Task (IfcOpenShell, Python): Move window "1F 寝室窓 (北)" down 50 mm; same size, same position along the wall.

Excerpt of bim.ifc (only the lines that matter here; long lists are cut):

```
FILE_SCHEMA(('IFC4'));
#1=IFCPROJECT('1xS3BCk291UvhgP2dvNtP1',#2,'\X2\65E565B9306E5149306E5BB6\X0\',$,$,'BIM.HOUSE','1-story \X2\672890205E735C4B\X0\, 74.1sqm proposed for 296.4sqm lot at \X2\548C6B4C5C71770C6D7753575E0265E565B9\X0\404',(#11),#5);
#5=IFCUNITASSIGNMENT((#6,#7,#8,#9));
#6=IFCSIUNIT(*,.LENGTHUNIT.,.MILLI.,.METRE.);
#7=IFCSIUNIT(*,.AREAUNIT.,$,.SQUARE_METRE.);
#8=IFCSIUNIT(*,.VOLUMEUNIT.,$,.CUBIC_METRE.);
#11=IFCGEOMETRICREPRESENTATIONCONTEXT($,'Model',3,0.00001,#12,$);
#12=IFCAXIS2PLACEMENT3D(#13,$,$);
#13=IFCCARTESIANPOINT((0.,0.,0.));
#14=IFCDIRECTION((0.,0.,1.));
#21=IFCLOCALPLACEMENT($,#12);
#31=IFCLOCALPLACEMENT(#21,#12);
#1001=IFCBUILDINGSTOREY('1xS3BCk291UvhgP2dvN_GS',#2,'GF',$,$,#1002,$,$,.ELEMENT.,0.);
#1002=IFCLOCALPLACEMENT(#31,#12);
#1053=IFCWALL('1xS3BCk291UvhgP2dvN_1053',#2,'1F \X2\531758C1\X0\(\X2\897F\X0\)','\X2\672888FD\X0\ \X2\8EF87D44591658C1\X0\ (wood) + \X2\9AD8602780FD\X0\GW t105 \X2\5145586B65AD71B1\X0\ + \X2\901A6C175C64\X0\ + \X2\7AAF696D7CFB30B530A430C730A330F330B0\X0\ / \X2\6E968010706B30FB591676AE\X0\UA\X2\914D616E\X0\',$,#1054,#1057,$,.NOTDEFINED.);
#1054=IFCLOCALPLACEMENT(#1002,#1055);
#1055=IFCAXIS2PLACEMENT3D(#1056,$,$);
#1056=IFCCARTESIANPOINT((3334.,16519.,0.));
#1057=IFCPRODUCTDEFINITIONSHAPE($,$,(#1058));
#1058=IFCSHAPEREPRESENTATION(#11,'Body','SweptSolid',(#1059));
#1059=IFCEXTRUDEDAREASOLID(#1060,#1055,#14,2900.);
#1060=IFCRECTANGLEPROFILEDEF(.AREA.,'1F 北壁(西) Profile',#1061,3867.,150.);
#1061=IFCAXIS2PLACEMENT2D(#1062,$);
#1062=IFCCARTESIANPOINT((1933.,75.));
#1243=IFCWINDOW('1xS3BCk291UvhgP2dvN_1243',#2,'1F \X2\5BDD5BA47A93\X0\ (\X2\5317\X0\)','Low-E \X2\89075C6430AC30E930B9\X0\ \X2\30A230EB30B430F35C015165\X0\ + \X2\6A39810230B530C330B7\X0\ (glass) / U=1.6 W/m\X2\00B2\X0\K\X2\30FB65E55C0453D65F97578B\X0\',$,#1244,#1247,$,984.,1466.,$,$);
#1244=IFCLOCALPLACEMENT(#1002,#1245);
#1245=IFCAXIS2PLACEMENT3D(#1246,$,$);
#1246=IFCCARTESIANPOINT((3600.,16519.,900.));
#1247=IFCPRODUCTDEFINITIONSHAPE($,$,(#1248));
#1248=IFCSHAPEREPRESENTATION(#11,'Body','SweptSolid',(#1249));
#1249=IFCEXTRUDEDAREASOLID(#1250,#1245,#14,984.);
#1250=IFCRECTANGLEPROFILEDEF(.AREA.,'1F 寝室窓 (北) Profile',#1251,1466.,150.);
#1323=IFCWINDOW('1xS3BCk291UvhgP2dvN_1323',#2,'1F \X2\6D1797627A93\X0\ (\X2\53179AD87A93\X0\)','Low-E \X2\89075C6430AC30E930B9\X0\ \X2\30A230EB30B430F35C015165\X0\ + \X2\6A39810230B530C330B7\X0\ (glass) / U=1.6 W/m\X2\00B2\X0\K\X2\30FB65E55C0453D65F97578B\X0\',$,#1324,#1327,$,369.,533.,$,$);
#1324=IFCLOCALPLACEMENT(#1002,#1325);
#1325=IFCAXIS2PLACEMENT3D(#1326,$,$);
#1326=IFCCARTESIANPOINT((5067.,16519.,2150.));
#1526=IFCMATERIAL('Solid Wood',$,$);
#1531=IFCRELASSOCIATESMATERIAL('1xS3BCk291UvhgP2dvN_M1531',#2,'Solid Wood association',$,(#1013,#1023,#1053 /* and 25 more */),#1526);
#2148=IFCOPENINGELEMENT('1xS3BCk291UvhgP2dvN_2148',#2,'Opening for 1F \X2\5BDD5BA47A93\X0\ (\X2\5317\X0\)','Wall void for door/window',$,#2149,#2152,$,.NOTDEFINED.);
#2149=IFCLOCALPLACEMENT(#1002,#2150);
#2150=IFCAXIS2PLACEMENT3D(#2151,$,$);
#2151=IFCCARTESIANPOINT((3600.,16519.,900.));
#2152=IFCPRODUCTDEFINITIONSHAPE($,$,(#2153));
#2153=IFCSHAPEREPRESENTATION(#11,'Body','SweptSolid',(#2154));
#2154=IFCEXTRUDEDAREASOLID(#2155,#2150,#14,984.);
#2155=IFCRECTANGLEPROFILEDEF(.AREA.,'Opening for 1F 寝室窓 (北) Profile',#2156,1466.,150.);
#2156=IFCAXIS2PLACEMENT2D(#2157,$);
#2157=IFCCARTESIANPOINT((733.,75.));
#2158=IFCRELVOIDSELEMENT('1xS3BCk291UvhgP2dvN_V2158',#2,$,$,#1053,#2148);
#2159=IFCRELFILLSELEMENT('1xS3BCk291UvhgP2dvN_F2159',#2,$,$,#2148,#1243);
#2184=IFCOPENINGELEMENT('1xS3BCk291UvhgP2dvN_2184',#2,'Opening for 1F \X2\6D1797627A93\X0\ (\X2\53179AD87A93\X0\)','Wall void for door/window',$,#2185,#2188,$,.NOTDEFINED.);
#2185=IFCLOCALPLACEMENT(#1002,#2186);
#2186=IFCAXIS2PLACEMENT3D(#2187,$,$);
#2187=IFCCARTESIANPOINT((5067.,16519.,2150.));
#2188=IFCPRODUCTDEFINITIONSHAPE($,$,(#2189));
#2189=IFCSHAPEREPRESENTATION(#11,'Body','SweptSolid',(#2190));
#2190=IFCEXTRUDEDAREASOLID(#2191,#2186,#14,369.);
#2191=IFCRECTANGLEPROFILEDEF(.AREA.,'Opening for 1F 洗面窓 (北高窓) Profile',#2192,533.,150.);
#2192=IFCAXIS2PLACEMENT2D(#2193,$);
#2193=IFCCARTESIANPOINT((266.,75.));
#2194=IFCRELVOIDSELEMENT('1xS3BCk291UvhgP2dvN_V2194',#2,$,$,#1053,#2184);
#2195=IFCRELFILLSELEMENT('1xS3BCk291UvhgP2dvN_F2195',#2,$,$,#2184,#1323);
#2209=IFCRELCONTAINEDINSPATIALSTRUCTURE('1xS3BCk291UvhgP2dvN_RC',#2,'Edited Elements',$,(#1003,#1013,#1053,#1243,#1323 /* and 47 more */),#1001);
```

```python
import numpy as np
import ifcopenshell
import ifcopenshell.api.geometry
import ifcopenshell.util.placement
import ifcopenshell.util.unit

model = ifcopenshell.open("bim.ifc")
unit_scale = ifcopenshell.util.unit.calculate_unit_scale(model)

window = model.by_guid("1xS3BCk291UvhgP2dvN_1243")
opening = window.FillsVoids[0].RelatingOpeningElement
dz = -0.05 / unit_scale

shift = np.array([0.0, 0.0, dz])
# The window is not placed relative to its opening, so move both.
for product in (opening, window):
    matrix = ifcopenshell.util.placement.get_local_placement(product.ObjectPlacement)
    matrix[:3, 3] += shift
    ifcopenshell.api.geometry.edit_object_placement(model, product=product, matrix=matrix, is_si=False)

print(f"moved by {dz * unit_scale:+.3f} m")

model.write("bim_v2.ifc")
```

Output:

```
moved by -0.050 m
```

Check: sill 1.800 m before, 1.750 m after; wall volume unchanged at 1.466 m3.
